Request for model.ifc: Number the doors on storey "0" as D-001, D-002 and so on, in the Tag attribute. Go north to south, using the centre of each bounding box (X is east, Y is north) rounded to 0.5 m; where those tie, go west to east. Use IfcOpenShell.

First a look at what the model holds.

```python
import ifcopenshell
import ifcopenshell.util.element
import ifcopenshell.util.placement

model = ifcopenshell.open("model.ifc")
print(model.schema)
storey = next(s for s in model.by_type("IfcBuildingStorey") if s.Name == "0")
doors = [e for e in ifcopenshell.util.element.get_decomposition(storey) if e.is_a("IfcDoor")]
for e in sorted(doors, key=lambda e: e.id()):
    origin = ifcopenshell.util.placement.get_local_placement(e.ObjectPlacement)[:3, 3]
    print(e.id(), e.Tag, e.Name, origin.round(2) + 0.0, sep=" | ")
```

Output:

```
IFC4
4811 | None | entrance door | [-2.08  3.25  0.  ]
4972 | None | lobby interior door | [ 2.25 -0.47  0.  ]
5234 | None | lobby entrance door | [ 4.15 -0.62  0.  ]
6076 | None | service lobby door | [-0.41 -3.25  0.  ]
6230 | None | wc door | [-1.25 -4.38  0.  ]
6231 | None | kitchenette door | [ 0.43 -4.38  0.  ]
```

```python
import ifcopenshell
import ifcopenshell.geom
import ifcopenshell.util.element
import ifcopenshell.util.shape

model = ifcopenshell.open("model.ifc")
settings = ifcopenshell.geom.settings()
settings.set("use-world-coords", True)


def centre(element):
    shape = ifcopenshell.geom.create_shape(settings, element)
    return ifcopenshell.util.shape.get_bbox_centroid(shape.geometry)


storey = next(s for s in model.by_type("IfcBuildingStorey") if s.Name == "0")
doors = [e for e in ifcopenshell.util.element.get_decomposition(storey) if e.is_a("IfcDoor")]

# Insertion points can sit at a corner or the storey origin, so sort by the geometry (in metres).
centres = {e: centre(e) for e in doors}
doors.sort(key=lambda e: (-round(centres[e][1] / 0.5), centres[e][0]))

for i, e in enumerate(doors, start=1):
    number = f"D-0{i:02d}"
    e.Tag = number
    print(e.id(), number)

model.write("model_edited.ifc")
```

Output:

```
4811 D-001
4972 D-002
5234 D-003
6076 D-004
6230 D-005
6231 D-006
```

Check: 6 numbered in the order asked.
